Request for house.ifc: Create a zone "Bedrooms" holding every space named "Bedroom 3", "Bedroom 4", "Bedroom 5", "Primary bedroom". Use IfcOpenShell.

First a look at what the model holds.

```python
import ifcopenshell

model = ifcopenshell.open("house.ifc")
print(model.schema)
seen = {}
for space in model.by_type("IfcSpace"):
    seen[space.LongName] = seen.get(space.LongName, 0) + 1
for name, count in sorted(seen.items(), key=str):
    print(count, "x", name)
print("zones:", [z.Name for z in model.by_type("IfcZone")][:20])
```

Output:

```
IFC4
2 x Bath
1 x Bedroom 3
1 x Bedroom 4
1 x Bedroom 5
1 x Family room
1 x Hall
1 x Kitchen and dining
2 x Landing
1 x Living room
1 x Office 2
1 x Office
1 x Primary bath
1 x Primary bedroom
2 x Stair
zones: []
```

```python
import ifcopenshell
import ifcopenshell.api.group
import ifcopenshell.api.root

model = ifcopenshell.open("house.ifc")

names = {"Bedroom 3", "Bedroom 4", "Bedroom 5", "Primary bedroom"}
spaces = [s for s in model.by_type("IfcSpace") if s.LongName in names]

zone = ifcopenshell.api.root.create_entity(model, ifc_class="IfcZone", name="Bedrooms")
ifcopenshell.api.group.assign_group(model, products=spaces, group=zone)
print(len(spaces), "spaces in", zone.Name)

model.write("house_edited.ifc")
```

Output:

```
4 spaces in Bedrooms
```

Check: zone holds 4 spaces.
